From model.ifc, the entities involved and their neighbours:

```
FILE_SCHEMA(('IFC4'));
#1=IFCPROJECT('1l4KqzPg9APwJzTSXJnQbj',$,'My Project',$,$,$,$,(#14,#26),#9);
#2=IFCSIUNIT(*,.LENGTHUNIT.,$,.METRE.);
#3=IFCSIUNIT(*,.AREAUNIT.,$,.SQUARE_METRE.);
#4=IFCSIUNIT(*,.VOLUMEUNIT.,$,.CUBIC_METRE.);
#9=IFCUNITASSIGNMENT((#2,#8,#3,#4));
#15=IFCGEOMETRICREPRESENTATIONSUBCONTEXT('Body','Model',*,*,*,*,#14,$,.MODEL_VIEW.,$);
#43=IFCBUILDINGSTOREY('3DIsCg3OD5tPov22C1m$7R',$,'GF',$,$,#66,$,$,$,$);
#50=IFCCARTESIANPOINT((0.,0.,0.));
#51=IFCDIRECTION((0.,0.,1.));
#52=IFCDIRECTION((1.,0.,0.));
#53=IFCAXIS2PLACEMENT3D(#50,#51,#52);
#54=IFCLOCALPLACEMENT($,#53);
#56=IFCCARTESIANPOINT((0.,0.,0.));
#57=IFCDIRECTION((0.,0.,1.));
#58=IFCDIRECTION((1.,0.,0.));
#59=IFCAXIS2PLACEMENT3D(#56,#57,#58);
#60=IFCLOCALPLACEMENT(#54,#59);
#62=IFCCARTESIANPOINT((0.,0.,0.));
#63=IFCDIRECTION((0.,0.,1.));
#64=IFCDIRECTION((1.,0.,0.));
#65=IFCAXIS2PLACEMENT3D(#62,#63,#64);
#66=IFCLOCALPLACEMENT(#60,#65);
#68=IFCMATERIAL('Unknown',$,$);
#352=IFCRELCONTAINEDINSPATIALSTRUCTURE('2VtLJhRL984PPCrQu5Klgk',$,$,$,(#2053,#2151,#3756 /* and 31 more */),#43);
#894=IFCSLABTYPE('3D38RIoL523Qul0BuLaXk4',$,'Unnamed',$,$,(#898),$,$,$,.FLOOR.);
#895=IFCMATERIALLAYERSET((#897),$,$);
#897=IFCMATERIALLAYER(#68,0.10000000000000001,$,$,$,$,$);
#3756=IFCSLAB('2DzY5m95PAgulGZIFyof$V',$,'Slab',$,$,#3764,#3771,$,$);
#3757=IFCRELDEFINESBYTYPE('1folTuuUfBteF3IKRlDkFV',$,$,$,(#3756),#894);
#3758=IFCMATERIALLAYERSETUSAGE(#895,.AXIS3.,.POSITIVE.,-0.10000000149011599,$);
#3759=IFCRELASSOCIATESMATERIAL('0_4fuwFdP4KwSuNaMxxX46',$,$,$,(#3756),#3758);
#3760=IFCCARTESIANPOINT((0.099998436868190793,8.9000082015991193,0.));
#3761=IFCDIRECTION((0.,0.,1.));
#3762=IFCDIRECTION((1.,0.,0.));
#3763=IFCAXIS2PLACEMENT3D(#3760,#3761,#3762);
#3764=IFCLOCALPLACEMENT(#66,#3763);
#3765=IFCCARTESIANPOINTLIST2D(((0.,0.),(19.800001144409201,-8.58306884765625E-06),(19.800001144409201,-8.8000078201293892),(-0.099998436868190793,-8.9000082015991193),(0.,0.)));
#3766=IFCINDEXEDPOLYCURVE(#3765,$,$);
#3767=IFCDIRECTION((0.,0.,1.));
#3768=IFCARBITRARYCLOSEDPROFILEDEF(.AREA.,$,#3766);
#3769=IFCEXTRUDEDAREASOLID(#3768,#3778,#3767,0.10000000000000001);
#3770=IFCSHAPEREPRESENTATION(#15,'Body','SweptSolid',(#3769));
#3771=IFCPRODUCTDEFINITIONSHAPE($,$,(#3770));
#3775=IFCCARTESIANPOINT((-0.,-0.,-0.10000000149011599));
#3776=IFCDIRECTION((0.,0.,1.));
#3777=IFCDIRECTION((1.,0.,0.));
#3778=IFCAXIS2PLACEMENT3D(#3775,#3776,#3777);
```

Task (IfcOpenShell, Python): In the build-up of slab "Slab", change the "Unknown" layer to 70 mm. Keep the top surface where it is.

```python
import ifcopenshell
import ifcopenshell.util.element
import ifcopenshell.util.representation

model = ifcopenshell.open("model.ifc")

layer_set = model.by_id(895)
layer = next(l for l in layer_set.MaterialLayers if l.Material and l.Material.Name == "Unknown")
change = 0.07 - layer.LayerThickness
layer.LayerThickness += change

# Geometry does not follow the layer set by itself.
slabs = [e for e in ifcopenshell.util.element.get_elements_by_material(model, layer_set) if e.is_a("IfcSlab")]
for slab in sorted(slabs, key=lambda e: e.id()):
    body = ifcopenshell.util.representation.get_representation(slab, "Model", "Body")
    solid = body.Items[0]
    old_depth = solid.Depth
    solid.Depth += change
    # Extruded upwards: lower the start of the extrusion so the top stays.
    x, y, z = solid.Position.Location.Coordinates
    solid.Position.Location = model.createIfcCartesianPoint((x, y, z - change))
    print(slab.id(), f"{old_depth:g} -> {solid.Depth:g}")

# The layers are counted up from the underside, which has moved.
for usage in {ifcopenshell.util.element.get_material(slab) for slab in slabs}:
    usage.OffsetFromReferenceLine -= change

model.write("model_rev.ifc")
```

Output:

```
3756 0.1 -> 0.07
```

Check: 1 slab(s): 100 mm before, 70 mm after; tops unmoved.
